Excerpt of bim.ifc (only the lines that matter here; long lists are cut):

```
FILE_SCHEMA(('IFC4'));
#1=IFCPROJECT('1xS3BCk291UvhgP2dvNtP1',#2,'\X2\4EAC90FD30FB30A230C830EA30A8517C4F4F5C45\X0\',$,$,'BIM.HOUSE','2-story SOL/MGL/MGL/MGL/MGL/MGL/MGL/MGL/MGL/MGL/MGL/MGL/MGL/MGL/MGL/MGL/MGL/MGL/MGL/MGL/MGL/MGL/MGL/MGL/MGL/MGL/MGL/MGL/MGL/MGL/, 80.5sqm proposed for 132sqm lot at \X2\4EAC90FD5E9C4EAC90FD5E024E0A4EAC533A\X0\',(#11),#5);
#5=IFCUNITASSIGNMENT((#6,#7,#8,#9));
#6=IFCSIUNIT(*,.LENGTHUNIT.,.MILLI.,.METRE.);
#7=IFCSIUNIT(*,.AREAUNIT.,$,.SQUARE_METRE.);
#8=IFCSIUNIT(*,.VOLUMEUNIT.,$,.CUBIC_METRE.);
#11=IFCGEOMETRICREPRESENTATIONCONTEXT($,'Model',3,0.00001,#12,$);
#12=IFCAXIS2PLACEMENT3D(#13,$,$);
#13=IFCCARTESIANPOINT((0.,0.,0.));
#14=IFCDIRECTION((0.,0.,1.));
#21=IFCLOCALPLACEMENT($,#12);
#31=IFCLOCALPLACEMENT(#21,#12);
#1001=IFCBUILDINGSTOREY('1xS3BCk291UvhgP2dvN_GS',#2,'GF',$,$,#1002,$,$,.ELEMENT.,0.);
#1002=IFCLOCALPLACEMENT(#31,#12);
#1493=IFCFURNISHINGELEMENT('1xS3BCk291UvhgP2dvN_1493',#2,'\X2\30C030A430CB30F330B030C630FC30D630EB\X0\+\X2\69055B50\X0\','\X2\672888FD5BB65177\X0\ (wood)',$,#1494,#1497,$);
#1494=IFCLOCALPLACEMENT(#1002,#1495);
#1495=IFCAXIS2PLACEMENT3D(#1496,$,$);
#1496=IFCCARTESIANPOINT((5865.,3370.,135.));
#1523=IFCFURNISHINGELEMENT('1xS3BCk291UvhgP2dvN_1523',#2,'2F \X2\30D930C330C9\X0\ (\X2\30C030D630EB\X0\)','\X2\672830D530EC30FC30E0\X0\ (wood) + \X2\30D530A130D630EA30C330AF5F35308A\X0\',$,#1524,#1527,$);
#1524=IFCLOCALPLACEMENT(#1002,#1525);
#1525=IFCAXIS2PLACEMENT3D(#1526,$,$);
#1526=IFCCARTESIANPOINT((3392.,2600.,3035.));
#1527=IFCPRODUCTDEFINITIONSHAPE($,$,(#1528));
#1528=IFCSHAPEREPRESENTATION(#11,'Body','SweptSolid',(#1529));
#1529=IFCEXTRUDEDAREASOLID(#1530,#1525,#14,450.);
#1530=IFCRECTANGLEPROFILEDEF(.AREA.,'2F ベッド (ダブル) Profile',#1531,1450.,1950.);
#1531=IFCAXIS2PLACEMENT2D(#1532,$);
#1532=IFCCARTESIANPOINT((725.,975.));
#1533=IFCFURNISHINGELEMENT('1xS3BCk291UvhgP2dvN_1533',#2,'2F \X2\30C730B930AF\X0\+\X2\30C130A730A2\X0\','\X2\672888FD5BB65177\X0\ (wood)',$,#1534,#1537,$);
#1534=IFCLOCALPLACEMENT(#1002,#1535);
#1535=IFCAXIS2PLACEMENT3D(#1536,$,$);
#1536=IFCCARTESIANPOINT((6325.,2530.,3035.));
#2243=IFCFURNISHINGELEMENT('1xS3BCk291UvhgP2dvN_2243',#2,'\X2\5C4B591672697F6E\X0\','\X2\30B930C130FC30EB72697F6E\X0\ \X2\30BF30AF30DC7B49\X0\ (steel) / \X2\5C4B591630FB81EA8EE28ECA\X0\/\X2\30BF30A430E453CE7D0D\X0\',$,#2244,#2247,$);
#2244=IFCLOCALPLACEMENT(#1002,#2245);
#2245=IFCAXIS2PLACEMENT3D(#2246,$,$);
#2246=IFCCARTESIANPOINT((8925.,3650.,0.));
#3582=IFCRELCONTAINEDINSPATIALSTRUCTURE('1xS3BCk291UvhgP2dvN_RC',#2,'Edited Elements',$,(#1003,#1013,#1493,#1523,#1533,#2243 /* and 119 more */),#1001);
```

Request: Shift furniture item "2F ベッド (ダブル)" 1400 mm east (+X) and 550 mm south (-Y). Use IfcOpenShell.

```python
import ifcopenshell
import ifcopenshell.api.geometry
import ifcopenshell.util.placement
import ifcopenshell.util.unit

model = ifcopenshell.open("bim.ifc")
unit_scale = ifcopenshell.util.unit.calculate_unit_scale(model)

item = model.by_guid("1xS3BCk291UvhgP2dvN_1523")
matrix = ifcopenshell.util.placement.get_local_placement(item.ObjectPlacement)
matrix[0, 3] += 1.4 / unit_scale
matrix[1, 3] -= 0.55 / unit_scale
ifcopenshell.api.geometry.edit_object_placement(model, product=item, matrix=matrix, is_si=False)

print(ifcopenshell.util.placement.get_local_placement(item.ObjectPlacement).round(3) + 0.0)

model.write("bim-out.ifc")
```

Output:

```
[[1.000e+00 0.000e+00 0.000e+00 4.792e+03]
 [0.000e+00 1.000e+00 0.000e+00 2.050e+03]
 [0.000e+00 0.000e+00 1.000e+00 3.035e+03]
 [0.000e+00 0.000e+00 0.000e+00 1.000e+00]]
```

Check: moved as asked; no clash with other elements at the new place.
